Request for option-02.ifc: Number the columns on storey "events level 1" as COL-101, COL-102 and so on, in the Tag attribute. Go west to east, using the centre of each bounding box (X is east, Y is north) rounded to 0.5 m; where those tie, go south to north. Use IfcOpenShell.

First a look at what the model holds.

```python
import ifcopenshell
import ifcopenshell.util.element
import ifcopenshell.util.placement

model = ifcopenshell.open("option-02.ifc")
print(model.schema)
storey = next(s for s in model.by_type("IfcBuildingStorey") if s.Name == "events level 1")
columns = [e for e in ifcopenshell.util.element.get_decomposition(storey) if e.is_a("IfcColumn")]
for e in sorted(columns, key=lambda e: e.id()):
    origin = ifcopenshell.util.placement.get_local_placement(e.ObjectPlacement)[:3, 3]
    print(e.id(), e.Tag, e.Name, origin.round(2) + 0.0, sep=" | ")
```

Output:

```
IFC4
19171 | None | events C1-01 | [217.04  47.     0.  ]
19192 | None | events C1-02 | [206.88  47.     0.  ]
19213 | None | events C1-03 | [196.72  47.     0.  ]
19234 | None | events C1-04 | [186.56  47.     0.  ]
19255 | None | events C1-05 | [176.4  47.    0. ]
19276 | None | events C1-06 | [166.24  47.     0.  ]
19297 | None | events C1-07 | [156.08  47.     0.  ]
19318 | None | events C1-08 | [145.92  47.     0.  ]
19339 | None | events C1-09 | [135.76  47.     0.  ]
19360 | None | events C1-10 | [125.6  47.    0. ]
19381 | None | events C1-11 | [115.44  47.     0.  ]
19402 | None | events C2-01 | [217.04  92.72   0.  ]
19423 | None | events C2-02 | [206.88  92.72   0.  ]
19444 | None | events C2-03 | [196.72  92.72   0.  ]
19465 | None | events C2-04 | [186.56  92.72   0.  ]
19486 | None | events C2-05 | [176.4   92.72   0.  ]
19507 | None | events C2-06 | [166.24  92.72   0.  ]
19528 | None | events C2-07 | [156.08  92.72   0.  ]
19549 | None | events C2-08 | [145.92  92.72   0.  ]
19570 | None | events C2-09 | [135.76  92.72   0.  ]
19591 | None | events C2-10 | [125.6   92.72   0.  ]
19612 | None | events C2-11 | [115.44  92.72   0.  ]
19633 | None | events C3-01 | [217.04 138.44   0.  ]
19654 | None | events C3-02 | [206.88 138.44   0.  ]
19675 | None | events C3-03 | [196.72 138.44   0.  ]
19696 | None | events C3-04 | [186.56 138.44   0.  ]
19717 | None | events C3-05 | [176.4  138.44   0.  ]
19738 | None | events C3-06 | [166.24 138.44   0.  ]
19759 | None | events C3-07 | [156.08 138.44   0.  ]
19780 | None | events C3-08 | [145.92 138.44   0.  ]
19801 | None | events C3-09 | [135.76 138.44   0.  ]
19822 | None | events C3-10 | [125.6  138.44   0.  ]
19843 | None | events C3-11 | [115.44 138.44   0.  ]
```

```python
import ifcopenshell
import ifcopenshell.geom
import ifcopenshell.util.element
import ifcopenshell.util.shape

model = ifcopenshell.open("option-02.ifc")
settings = ifcopenshell.geom.settings()
settings.set("use-world-coords", True)


def centre(element):
    shape = ifcopenshell.geom.create_shape(settings, element)
    return ifcopenshell.util.shape.get_bbox_centroid(shape.geometry)


storey = next(s for s in model.by_type("IfcBuildingStorey") if s.Name == "events level 1")
columns = [e for e in ifcopenshell.util.element.get_decomposition(storey) if e.is_a("IfcColumn")]

# Insertion points can sit at a corner or the storey origin, so sort by the geometry (in metres).
centres = {e: centre(e) for e in columns}
columns.sort(key=lambda e: (round(centres[e][0] / 0.5), centres[e][1]))

for i, e in enumerate(columns, start=1):
    number = f"COL-1{i:02d}"
    e.Tag = number
    print(e.id(), number)

model.write("option-02_edited.ifc")
```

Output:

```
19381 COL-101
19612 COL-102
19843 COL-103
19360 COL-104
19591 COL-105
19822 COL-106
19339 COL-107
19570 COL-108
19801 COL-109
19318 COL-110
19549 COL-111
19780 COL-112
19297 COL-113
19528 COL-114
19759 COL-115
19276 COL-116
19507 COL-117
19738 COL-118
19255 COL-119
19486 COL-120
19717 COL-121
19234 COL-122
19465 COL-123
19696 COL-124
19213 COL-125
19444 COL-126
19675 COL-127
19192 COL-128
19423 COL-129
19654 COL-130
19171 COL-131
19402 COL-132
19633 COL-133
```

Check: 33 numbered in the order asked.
